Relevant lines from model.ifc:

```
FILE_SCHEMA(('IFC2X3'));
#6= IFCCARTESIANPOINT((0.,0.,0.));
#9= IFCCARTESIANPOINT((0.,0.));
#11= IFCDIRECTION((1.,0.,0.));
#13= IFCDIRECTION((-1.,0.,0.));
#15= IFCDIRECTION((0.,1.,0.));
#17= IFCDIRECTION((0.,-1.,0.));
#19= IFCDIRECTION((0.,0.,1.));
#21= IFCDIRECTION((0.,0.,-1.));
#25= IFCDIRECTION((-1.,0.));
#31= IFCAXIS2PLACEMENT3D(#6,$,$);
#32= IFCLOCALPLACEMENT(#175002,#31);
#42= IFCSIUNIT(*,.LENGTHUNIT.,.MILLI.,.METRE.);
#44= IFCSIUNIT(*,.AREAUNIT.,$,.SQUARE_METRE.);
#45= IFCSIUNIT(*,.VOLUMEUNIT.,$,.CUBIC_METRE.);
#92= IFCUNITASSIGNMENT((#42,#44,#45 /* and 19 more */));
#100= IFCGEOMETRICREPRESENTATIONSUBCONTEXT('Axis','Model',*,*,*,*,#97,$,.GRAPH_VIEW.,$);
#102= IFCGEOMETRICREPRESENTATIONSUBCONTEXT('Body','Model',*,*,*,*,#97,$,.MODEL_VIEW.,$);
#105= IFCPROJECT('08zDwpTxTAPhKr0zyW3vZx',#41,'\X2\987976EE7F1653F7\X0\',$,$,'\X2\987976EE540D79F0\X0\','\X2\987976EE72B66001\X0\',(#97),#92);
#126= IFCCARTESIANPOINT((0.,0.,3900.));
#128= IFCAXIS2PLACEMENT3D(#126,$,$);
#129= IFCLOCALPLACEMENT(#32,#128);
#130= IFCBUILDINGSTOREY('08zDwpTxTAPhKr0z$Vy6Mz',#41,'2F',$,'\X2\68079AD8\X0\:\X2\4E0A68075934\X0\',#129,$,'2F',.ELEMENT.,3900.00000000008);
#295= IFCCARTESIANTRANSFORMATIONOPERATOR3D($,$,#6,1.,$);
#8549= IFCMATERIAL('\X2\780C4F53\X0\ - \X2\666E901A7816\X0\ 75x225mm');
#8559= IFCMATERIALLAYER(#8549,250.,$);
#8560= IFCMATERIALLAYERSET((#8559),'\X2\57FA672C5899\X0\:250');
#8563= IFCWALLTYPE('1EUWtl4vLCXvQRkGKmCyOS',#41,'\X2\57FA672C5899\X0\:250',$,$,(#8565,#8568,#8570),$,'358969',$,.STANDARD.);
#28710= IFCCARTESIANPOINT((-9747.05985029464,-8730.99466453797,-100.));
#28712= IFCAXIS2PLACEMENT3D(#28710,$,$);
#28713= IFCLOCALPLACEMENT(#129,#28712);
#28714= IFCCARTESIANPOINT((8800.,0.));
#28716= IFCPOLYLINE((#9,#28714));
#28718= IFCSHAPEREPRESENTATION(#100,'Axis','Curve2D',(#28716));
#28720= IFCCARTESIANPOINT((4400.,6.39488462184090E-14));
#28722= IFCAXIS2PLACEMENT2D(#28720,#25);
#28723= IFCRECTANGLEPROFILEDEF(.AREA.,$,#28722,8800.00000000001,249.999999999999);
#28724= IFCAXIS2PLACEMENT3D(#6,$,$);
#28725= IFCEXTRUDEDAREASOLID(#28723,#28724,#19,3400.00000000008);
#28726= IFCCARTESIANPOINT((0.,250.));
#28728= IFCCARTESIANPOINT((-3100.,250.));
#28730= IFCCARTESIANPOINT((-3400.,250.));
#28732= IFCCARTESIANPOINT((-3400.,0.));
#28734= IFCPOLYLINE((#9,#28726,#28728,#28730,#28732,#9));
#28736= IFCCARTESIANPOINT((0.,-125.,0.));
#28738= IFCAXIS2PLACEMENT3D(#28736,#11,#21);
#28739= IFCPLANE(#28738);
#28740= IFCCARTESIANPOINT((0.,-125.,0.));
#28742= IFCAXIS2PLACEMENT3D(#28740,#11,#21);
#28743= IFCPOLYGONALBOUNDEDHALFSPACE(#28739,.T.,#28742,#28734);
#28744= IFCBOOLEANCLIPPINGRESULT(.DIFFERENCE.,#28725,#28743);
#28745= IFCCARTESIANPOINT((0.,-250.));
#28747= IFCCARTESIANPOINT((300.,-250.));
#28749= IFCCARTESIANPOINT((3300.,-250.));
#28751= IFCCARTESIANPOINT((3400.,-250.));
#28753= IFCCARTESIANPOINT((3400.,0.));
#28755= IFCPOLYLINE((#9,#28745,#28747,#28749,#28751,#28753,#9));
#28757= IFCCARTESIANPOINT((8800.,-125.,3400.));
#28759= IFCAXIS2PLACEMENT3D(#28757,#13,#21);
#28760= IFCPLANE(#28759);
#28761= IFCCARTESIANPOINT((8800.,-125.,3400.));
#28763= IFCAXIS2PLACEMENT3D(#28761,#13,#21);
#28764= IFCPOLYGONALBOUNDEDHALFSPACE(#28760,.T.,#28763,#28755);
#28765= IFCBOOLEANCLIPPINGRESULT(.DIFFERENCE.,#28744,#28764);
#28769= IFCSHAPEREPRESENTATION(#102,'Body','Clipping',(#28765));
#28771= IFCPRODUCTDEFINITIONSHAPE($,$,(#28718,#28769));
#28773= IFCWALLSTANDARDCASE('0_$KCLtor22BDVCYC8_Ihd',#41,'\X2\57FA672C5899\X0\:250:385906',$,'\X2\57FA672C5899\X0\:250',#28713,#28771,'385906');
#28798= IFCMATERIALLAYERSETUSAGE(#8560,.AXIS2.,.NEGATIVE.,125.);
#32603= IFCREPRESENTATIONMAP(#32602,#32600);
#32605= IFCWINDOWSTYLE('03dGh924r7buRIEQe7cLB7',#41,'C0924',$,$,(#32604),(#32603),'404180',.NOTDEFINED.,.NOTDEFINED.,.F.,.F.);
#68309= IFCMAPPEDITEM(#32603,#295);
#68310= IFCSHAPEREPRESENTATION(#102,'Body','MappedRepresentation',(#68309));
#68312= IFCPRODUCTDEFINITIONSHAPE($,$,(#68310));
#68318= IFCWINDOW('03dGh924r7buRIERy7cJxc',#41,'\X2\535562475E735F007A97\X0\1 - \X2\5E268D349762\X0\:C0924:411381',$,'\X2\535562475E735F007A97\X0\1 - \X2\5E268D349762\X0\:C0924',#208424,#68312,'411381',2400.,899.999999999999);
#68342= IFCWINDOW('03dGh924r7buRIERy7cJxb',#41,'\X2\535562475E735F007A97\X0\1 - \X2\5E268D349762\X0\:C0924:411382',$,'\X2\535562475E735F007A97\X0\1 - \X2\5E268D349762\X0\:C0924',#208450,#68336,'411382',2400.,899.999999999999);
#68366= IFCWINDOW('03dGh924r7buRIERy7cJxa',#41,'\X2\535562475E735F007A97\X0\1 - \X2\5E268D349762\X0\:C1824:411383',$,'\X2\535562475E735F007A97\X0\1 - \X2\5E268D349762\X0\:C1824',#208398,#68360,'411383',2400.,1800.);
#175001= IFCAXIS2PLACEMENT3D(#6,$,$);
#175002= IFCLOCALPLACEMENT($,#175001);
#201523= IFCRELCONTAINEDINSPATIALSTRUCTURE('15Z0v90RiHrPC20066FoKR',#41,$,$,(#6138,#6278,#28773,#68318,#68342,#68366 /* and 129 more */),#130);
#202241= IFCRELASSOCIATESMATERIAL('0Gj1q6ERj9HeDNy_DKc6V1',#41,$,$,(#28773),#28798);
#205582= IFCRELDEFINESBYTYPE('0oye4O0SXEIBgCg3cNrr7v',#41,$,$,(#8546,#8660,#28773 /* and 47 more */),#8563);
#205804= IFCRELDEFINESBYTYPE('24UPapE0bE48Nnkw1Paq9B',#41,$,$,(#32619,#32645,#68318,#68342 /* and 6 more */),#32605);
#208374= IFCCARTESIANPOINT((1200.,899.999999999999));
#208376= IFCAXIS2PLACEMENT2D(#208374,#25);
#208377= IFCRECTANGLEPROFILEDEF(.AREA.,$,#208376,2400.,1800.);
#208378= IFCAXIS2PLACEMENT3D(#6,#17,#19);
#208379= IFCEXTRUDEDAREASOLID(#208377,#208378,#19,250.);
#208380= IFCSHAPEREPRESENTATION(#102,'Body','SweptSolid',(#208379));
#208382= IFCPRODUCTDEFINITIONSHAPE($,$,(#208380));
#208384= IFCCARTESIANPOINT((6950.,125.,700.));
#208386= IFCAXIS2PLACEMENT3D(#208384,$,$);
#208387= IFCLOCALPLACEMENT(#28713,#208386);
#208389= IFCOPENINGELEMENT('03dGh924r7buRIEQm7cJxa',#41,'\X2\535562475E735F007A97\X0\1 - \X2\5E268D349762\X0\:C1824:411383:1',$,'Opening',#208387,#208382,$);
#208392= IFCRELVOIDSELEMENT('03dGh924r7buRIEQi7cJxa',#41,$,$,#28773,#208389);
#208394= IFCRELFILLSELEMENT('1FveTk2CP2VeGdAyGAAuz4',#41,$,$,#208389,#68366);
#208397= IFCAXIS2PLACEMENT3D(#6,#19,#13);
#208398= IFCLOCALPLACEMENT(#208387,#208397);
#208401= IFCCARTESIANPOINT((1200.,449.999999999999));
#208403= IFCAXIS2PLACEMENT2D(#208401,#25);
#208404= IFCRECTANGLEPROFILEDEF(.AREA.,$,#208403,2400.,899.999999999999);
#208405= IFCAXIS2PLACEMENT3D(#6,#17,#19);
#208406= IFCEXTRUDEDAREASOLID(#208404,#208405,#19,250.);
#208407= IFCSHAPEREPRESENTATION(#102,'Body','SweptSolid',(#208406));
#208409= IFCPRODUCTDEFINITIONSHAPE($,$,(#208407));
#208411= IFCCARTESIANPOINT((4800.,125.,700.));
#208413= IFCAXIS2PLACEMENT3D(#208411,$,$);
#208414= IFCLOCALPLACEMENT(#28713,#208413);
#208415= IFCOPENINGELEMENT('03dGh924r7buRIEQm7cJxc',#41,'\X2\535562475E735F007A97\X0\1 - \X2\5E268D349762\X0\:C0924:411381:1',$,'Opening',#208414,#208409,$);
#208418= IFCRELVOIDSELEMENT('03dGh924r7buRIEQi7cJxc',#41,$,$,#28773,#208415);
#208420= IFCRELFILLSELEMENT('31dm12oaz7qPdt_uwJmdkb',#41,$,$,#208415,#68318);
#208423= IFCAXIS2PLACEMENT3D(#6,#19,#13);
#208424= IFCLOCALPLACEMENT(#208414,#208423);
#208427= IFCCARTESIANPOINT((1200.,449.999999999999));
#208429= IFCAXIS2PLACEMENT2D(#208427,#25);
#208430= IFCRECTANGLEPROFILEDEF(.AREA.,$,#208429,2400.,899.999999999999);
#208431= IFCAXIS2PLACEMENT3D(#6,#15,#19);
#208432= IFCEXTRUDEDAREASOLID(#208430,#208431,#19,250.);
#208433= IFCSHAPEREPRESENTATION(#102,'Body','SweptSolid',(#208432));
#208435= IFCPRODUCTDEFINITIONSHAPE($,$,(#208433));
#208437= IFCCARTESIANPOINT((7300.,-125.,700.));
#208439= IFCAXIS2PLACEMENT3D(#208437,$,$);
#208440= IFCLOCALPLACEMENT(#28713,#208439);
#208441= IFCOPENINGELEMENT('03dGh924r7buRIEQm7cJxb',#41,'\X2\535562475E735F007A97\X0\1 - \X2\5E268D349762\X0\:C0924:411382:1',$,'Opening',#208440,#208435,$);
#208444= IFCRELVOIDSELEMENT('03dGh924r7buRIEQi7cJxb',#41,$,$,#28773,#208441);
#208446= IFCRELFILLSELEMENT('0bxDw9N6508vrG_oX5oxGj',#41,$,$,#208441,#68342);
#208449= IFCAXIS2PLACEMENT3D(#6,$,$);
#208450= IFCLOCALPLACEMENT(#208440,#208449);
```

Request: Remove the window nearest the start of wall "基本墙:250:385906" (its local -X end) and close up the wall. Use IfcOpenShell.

```python
import ifcopenshell
import ifcopenshell.api.feature
import ifcopenshell.api.root
import ifcopenshell.geom
import ifcopenshell.util.shape

model = ifcopenshell.open("model.ifc")
settings = ifcopenshell.geom.settings()


def volume(element):
    """Net volume in cubic metres, openings subtracted."""
    shape = ifcopenshell.geom.create_shape(settings, element)
    return ifcopenshell.util.shape.get_volume(shape.geometry)


window = model.by_guid("03dGh924r7buRIERy7cJxc")
opening = window.FillsVoids[0].RelatingOpeningElement
wall = opening.VoidsElements[0].RelatingBuildingElement
before = volume(wall)

ifcopenshell.api.root.remove_product(model, product=window)
ifcopenshell.api.feature.remove_feature(model, feature=opening)

after = volume(wall)

print(f"wall volume {before:.3f} -> {after:.3f} m3")

model.write("model_edited.ifc")
```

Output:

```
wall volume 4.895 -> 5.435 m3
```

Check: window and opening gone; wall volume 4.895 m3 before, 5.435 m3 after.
